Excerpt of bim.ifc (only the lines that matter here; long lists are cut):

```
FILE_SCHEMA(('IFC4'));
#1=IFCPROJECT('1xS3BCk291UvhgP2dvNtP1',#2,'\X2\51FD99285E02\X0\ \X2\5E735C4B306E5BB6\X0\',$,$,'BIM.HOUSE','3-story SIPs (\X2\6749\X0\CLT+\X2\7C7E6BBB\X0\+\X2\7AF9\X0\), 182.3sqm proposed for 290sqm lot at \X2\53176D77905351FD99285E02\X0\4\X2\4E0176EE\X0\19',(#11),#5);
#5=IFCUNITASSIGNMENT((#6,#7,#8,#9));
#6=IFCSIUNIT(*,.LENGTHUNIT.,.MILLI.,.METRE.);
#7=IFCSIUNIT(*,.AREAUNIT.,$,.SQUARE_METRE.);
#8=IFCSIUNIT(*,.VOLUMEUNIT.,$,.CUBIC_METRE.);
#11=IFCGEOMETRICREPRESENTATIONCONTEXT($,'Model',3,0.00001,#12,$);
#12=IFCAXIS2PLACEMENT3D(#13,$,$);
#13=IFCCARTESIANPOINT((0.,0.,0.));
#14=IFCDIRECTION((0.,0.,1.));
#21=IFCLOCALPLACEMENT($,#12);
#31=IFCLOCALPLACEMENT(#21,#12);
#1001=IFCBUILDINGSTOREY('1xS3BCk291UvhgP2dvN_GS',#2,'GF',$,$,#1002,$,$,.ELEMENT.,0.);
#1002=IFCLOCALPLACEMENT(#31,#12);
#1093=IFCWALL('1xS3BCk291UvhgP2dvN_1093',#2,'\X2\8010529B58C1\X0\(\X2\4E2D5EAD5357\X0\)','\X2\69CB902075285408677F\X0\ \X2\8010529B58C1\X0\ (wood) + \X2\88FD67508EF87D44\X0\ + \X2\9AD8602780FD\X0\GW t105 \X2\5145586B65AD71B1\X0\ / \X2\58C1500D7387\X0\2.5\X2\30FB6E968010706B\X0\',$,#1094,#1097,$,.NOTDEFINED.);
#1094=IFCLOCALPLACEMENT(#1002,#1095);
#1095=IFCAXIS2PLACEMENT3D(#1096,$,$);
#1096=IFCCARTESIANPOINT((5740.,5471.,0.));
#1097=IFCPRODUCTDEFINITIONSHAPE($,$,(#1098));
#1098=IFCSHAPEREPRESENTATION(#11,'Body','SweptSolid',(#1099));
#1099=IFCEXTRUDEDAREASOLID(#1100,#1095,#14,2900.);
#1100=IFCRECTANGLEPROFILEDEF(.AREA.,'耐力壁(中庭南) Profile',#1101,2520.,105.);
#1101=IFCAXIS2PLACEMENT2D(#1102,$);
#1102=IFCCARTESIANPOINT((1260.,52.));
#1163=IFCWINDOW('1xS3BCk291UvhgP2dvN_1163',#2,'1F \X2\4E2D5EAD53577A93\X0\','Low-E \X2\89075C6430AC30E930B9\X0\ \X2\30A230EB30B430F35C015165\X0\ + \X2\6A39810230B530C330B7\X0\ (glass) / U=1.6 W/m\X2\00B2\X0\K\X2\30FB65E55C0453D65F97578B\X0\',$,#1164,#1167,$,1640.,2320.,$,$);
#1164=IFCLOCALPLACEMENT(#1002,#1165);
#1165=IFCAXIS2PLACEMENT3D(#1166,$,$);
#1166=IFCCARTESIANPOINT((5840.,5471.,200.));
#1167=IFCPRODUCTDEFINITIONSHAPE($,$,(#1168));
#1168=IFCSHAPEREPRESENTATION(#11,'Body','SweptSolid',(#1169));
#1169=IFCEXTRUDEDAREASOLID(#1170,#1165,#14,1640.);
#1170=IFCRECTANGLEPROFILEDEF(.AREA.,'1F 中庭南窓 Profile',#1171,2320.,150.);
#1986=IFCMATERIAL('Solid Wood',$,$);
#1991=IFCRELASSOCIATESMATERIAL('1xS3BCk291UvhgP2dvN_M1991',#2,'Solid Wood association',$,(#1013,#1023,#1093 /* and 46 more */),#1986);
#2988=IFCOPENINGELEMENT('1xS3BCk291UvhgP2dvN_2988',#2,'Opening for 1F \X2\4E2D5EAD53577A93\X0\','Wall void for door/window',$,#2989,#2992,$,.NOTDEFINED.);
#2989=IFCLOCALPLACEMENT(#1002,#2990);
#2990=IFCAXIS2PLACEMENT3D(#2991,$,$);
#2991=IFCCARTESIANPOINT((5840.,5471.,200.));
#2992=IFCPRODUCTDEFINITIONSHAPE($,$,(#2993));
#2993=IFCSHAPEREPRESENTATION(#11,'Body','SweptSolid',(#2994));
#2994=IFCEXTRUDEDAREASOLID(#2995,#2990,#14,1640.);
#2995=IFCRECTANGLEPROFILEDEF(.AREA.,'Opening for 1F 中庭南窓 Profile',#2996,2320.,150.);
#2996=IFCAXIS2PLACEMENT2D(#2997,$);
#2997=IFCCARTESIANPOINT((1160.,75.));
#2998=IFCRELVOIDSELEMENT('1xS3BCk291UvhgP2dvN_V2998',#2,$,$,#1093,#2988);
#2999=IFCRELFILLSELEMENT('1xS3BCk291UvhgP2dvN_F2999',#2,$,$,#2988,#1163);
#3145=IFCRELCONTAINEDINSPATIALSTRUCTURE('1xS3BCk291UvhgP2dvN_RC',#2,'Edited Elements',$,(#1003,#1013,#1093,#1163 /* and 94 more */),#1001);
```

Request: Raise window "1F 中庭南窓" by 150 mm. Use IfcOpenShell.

```python
import numpy as np
import ifcopenshell
import ifcopenshell.api.geometry
import ifcopenshell.util.placement
import ifcopenshell.util.unit

model = ifcopenshell.open("bim.ifc")
unit_scale = ifcopenshell.util.unit.calculate_unit_scale(model)

window = model.by_guid("1xS3BCk291UvhgP2dvN_1163")
opening = window.FillsVoids[0].RelatingOpeningElement
dz = 150.0

shift = np.array([0.0, 0.0, dz])
# The window is not placed relative to its opening, so move both.
for product in (opening, window):
    matrix = ifcopenshell.util.placement.get_local_placement(product.ObjectPlacement)
    matrix[:3, 3] += shift
    ifcopenshell.api.geometry.edit_object_placement(model, product=product, matrix=matrix, is_si=False)

print(f"moved by {dz * unit_scale:+.3f} m")

model.write("bim_edited.ifc")
```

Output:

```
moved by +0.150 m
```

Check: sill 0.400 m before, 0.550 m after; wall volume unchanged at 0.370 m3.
